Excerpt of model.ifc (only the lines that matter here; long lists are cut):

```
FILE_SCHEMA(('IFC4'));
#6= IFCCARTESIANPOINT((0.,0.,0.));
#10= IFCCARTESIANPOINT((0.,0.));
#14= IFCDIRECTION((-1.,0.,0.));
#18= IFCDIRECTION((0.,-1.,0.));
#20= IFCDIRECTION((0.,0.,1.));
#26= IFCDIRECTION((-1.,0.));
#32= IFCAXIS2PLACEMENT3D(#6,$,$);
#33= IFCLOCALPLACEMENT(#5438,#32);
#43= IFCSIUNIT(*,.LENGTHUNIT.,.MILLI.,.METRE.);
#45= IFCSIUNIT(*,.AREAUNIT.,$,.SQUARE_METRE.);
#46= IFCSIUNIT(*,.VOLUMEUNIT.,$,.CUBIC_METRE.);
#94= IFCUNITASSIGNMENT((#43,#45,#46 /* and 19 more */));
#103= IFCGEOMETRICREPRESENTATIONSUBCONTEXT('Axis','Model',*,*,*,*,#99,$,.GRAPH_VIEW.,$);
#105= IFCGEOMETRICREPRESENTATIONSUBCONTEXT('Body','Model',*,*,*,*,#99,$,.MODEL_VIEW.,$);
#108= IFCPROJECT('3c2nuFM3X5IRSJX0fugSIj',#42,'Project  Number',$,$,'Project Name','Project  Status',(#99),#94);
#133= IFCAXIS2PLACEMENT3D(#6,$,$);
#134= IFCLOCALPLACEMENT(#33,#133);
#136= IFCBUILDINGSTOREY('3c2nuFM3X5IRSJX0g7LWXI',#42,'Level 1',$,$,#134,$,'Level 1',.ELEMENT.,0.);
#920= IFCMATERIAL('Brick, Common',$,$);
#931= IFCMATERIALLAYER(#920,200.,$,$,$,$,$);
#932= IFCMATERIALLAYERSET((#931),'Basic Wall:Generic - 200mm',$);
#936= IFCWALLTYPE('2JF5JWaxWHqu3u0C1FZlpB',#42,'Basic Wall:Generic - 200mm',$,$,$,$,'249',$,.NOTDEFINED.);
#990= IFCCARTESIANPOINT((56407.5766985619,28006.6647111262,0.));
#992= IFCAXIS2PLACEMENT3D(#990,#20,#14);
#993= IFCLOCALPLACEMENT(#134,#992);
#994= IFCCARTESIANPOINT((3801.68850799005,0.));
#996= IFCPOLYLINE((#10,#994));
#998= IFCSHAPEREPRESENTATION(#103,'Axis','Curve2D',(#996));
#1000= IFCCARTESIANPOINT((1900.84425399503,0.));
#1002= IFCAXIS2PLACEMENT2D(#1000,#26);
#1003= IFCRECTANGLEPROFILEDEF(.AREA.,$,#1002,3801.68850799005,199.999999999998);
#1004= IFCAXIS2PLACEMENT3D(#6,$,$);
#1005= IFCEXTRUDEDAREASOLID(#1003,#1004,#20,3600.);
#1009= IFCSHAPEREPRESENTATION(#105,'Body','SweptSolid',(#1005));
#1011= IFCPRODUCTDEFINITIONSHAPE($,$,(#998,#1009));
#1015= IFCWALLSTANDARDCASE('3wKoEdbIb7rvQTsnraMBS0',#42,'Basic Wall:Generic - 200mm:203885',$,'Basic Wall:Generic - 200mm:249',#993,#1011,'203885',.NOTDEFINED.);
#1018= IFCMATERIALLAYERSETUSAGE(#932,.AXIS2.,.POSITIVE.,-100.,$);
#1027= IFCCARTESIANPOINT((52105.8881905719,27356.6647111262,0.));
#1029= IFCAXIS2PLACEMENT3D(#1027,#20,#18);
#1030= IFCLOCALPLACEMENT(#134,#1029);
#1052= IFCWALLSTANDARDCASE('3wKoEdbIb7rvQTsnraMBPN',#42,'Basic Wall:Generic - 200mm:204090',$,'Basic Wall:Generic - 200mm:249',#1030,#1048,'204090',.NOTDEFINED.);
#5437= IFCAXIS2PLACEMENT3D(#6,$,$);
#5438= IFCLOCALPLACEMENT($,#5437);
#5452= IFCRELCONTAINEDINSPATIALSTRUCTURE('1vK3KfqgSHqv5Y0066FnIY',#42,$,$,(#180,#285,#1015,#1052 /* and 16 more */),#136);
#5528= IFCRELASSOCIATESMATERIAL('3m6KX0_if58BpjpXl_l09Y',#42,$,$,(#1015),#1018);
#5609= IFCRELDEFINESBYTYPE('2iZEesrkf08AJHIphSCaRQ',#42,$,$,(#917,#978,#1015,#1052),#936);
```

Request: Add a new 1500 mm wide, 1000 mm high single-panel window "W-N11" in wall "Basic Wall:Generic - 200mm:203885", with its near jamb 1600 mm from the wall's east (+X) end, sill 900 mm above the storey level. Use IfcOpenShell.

```python
import numpy as np
import ifcopenshell
import ifcopenshell.api.feature
import ifcopenshell.api.geometry
import ifcopenshell.api.root
import ifcopenshell.api.spatial
import ifcopenshell.geom
import ifcopenshell.util.element
import ifcopenshell.util.placement
import ifcopenshell.util.representation
import ifcopenshell.util.shape
import ifcopenshell.util.unit

model = ifcopenshell.open("model.ifc")
unit_scale = ifcopenshell.util.unit.calculate_unit_scale(model)
settings = ifcopenshell.geom.settings()


def volume(element):
    """Net volume in cubic metres, openings subtracted."""
    shape = ifcopenshell.geom.create_shape(settings, element)
    return ifcopenshell.util.shape.get_volume(shape.geometry)


wall = model.by_id(1015)
storey = ifcopenshell.util.element.get_container(wall, ifc_class="IfcBuildingStorey")
context = ifcopenshell.util.representation.get_context(model, "Model", "Body", "MODEL_VIEW")
before = volume(wall)

width, height, from_end, sill = 1.5, 1, 1.6, 0.9  # metres

# The wall runs along its own X axis, and the end named is its -X end.
wall_shape = ifcopenshell.geom.create_shape(settings, wall)
x, y, z = ifcopenshell.util.shape.get_vertices(wall_shape.geometry).T
start = x.min() + from_end
face, thickness = float(y.min()), float(y.max() - y.min())
wall_matrix = ifcopenshell.util.placement.get_local_placement(wall.ObjectPlacement)
level = ifcopenshell.util.placement.get_local_placement(storey.ObjectPlacement)[2, 3]


def in_wall(x, y):
    """Placement at x, y metres in the wall's axes, at sill height."""
    matrix = wall_matrix.copy()
    matrix[:, 3] = wall_matrix @ np.array([x / unit_scale, y / unit_scale, 0.0, 1.0])
    matrix[2, 3] = level + sill / unit_scale
    return matrix


# Opening: a box that overshoots both wall faces by 50 mm.
opening = ifcopenshell.api.root.create_entity(model, ifc_class="IfcOpeningElement", predefined_type="OPENING")
box = ifcopenshell.api.geometry.add_wall_representation(
    model, context=context, length=width, height=height, thickness=thickness + 0.1
)
ifcopenshell.api.geometry.assign_representation(model, product=opening, representation=box)
ifcopenshell.api.geometry.edit_object_placement(model, product=opening, matrix=in_wall(start, face - 0.05), is_si=False)
ifcopenshell.api.feature.add_feature(model, feature=opening, element=wall)

window = ifcopenshell.api.root.create_entity(model, ifc_class="IfcWindow", name="W-N11", predefined_type="WINDOW")
window.OverallWidth, window.OverallHeight = width / unit_scale, height / unit_scale
window.PartitioningType = "SINGLE_PANEL"
body = ifcopenshell.api.geometry.add_window_representation(
    model,
    context=context,
    overall_width=window.OverallWidth,
    overall_height=window.OverallHeight,
    partition_type="SINGLE_PANEL",
)
ifcopenshell.api.geometry.assign_representation(model, product=window, representation=body)
ifcopenshell.api.spatial.assign_container(model, products=[window], relating_structure=storey)
ifcopenshell.api.feature.add_filling(model, opening=opening, element=window)

# Centre the window in the wall's thickness.
ifcopenshell.api.geometry.edit_object_placement(model, product=window, matrix=in_wall(start, face), is_si=False)
window_shape = ifcopenshell.geom.create_shape(settings, window)
depth = ifcopenshell.util.shape.get_vertices(window_shape.geometry)[:, 1]
offset = face + thickness / 2 - (depth.min() + depth.max()) / 2
ifcopenshell.api.geometry.edit_object_placement(model, product=window, matrix=in_wall(start, offset), is_si=False)

after = volume(wall)

print(f"wall volume {before:.3f} -> {after:.3f} m3")

model.write("model_edited.ifc")
```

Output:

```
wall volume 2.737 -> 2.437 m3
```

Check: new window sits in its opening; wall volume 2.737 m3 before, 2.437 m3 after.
